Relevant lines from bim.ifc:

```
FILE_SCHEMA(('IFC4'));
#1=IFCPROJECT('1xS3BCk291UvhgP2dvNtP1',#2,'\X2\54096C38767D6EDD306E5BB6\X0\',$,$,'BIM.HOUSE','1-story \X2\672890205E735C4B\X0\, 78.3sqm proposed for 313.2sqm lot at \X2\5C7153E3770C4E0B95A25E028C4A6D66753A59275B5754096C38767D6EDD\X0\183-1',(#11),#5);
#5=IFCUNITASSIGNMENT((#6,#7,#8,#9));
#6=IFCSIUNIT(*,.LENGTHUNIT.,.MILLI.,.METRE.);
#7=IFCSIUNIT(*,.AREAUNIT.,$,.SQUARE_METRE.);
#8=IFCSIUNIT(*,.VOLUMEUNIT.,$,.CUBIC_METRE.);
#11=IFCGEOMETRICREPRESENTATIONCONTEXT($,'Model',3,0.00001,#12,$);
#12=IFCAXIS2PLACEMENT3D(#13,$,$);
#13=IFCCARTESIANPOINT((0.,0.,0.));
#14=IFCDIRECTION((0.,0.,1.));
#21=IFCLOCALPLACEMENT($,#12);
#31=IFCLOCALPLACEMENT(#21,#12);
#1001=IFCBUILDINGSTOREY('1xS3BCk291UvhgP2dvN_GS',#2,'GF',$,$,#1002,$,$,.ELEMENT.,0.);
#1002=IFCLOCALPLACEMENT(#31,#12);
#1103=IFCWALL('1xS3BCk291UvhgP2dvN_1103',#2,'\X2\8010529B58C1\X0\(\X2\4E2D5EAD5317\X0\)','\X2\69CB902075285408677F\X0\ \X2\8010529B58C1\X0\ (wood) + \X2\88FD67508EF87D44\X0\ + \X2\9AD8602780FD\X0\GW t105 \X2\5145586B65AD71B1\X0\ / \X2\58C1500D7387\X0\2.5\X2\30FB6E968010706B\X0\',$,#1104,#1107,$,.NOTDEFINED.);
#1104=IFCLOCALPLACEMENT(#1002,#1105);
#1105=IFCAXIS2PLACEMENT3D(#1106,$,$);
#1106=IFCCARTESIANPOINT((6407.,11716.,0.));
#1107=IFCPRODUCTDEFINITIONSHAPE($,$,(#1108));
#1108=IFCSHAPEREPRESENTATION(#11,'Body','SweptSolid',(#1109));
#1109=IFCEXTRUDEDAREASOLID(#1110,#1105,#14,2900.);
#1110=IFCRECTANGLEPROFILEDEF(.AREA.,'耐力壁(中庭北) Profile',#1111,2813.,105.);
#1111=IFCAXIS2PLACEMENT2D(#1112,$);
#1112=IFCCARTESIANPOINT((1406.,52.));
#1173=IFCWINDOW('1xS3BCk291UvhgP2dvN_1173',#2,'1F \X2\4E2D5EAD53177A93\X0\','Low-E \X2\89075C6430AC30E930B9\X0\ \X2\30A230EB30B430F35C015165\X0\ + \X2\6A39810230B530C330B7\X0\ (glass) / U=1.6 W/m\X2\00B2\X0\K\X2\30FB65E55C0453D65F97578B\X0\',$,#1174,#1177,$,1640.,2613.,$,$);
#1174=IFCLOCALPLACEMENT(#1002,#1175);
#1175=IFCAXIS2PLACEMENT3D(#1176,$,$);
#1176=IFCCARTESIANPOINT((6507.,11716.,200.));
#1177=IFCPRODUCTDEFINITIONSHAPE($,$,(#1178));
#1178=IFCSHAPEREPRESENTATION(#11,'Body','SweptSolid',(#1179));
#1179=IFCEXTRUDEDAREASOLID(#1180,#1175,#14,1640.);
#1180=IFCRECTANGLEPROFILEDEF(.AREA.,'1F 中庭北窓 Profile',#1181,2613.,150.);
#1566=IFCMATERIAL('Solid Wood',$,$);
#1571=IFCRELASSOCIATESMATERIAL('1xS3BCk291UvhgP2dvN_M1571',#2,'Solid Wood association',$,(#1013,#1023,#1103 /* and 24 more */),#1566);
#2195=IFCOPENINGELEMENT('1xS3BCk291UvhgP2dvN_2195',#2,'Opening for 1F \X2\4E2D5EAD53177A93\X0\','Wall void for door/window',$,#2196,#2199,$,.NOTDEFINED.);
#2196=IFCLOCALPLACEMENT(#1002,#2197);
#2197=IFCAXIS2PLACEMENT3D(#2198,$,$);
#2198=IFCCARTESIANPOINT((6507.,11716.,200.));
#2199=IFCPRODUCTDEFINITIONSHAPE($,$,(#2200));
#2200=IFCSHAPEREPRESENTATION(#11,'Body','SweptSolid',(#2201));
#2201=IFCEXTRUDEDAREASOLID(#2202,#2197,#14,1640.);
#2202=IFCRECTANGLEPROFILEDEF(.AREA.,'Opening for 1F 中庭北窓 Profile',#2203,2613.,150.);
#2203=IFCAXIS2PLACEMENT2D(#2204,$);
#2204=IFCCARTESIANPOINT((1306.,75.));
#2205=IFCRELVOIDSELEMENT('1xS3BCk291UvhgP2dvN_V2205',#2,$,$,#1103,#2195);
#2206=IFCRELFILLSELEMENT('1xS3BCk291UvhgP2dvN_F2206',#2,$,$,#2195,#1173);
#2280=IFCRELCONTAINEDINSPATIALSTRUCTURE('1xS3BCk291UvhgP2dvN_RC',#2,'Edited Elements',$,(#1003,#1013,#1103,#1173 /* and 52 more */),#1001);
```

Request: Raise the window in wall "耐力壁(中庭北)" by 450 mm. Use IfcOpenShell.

```python
import numpy as np
import ifcopenshell
import ifcopenshell.api.geometry
import ifcopenshell.util.placement
import ifcopenshell.util.unit

model = ifcopenshell.open("bim.ifc")
unit_scale = ifcopenshell.util.unit.calculate_unit_scale(model)

window = model.by_id(1173)
opening = window.FillsVoids[0].RelatingOpeningElement
dz = 0.45 / unit_scale

shift = np.array([0.0, 0.0, dz])
# The window is not placed relative to its opening, so move both.
for product in (opening, window):
    matrix = ifcopenshell.util.placement.get_local_placement(product.ObjectPlacement)
    matrix[:3, 3] += shift
    ifcopenshell.api.geometry.edit_object_placement(model, product=product, matrix=matrix, is_si=False)

print(f"moved by {dz * unit_scale:+.3f} m")

model.write("bim-out.ifc")
```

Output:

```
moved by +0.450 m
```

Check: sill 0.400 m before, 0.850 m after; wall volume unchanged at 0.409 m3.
